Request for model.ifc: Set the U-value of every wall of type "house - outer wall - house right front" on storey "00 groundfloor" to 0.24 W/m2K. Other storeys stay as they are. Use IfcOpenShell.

First a look at what the model holds.

```python
import ifcopenshell
import ifcopenshell.util.element

model = ifcopenshell.open("model.ifc")
print(model.schema)
storey = next(s for s in model.by_type("IfcBuildingStorey") if s.Name == "00 groundfloor")
walls = [e for e in ifcopenshell.util.element.get_decomposition(storey) if e.is_a("IfcWall")]
seen = {}
for e in walls:
    element_type = ifcopenshell.util.element.get_type(e)
    key = (element_type.Name if element_type != e and element_type else None, ifcopenshell.util.element.get_pset(e, "Pset_WallCommon", "ThermalTransmittance"))
    seen[key] = seen.get(key, 0) + 1
for (name, value), count in sorted(seen.items(), key=str):
    print(count, "x", name, "|", value)
```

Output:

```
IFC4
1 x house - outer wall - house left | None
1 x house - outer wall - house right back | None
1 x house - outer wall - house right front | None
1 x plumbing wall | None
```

```python
import ifcopenshell
import ifcopenshell.api.pset
import ifcopenshell.util.element

model = ifcopenshell.open("model.ifc")

storey = next(s for s in model.by_type("IfcBuildingStorey") if s.Name == "00 groundfloor")
walls = [e for e in ifcopenshell.util.element.get_decomposition(storey) if e.is_a("IfcWall")]

count = 0
for e in walls:
    element_type = ifcopenshell.util.element.get_type(e)
    if element_type in (None, e) or element_type.Name != "house - outer wall - house right front":
        continue
    # add_pset returns the element's existing set when there is one.
    pset = ifcopenshell.api.pset.add_pset(model, product=e, name="Pset_WallCommon")
    ifcopenshell.api.pset.edit_pset(model, pset=pset, properties={"ThermalTransmittance": 0.24})
    count += 1

print(count, "walls updated")

model.write("model_updated.ifc")
```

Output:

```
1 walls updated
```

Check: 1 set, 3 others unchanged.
